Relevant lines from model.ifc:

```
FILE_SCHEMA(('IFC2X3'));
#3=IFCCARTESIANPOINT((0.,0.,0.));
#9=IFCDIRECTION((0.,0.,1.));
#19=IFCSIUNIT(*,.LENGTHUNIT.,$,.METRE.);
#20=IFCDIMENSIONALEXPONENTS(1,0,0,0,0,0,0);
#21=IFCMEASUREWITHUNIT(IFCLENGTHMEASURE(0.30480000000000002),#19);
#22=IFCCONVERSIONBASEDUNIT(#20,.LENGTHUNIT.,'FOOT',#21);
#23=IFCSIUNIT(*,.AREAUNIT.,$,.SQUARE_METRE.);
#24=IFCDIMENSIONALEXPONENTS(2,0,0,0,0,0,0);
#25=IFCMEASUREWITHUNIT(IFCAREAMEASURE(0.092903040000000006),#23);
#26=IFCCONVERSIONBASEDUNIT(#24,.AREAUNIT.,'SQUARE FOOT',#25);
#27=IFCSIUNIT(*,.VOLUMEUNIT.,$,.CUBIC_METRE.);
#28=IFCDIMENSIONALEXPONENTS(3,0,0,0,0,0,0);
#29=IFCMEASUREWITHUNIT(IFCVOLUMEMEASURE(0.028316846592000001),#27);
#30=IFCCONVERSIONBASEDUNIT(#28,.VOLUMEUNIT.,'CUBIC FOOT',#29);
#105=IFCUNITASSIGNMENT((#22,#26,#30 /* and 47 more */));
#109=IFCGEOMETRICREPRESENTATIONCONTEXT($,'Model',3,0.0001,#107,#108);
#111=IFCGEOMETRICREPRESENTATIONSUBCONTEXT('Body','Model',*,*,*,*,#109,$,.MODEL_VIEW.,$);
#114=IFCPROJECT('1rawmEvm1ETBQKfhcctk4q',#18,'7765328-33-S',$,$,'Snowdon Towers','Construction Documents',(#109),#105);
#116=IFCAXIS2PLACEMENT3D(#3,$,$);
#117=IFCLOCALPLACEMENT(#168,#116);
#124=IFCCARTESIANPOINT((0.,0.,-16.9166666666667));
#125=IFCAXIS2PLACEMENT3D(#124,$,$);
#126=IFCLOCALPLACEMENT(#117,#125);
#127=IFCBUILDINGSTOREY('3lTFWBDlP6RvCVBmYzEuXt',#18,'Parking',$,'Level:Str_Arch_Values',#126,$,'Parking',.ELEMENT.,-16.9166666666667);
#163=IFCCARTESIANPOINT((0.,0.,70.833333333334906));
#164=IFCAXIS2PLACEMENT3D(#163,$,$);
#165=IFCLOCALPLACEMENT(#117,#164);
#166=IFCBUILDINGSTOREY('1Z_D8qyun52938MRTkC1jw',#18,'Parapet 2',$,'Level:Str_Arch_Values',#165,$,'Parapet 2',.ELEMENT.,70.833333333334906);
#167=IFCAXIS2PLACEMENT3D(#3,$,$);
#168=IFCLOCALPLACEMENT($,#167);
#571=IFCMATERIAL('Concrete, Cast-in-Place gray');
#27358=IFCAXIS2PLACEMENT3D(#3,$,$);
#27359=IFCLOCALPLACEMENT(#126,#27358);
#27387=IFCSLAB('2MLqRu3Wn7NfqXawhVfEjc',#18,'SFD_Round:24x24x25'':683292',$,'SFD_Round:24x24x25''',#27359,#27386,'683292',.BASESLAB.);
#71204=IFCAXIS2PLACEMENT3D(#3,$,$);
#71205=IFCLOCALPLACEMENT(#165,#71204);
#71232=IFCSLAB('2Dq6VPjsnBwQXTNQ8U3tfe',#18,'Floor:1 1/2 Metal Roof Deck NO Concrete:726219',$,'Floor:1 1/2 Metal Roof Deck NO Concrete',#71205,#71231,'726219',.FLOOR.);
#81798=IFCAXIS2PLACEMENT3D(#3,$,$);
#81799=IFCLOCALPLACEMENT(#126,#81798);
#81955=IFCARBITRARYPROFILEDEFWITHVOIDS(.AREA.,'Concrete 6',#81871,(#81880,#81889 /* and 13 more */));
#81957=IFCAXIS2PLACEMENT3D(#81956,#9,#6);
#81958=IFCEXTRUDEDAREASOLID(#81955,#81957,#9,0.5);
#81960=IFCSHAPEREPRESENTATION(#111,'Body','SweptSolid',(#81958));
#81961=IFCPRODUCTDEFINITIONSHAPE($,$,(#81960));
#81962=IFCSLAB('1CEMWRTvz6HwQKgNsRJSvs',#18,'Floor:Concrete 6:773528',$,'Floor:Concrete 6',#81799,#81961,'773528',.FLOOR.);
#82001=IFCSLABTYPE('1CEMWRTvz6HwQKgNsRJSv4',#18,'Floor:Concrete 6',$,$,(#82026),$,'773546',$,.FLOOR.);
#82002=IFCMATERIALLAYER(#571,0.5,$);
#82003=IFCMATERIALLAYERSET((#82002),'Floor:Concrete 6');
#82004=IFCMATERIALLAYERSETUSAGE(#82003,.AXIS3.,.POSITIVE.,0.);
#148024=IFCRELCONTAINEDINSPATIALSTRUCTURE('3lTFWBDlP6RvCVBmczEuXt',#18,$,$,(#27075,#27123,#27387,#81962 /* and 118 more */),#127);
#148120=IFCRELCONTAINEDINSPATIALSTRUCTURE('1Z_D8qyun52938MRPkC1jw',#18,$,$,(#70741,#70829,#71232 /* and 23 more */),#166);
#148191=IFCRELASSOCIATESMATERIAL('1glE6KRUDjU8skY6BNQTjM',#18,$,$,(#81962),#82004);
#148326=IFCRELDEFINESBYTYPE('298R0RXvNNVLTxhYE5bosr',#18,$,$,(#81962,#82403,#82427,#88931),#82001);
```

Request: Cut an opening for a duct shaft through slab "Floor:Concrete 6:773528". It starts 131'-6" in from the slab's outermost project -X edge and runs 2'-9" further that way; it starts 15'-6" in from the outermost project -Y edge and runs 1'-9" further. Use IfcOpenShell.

```python
import numpy as np
import ifcopenshell
import ifcopenshell.api.feature
import ifcopenshell.api.geometry
import ifcopenshell.api.root
import ifcopenshell.geom
import ifcopenshell.util.placement
import ifcopenshell.util.representation
import ifcopenshell.util.shape
import ifcopenshell.util.unit

model = ifcopenshell.open("model.ifc")
unit_scale = ifcopenshell.util.unit.calculate_unit_scale(model)
settings = ifcopenshell.geom.settings()


def volume(element):
    """Net volume in cubic metres, openings subtracted."""
    shape = ifcopenshell.geom.create_shape(settings, element)
    return ifcopenshell.util.shape.get_volume(shape.geometry)


slab = model.by_id(81962)
before = volume(slab)

# Extent in the slab's own axes, in metres. The edges named are its -X and -Y sides.
slab_shape = ifcopenshell.geom.create_shape(settings, slab)
vertices = ifcopenshell.util.shape.get_vertices(slab_shape.geometry)
x_min, y_min, bottom = vertices.min(axis=0)
top = vertices[:, 2].max()

opening = ifcopenshell.api.root.create_entity(model, ifc_class="IfcOpeningElement", name="Duct shaft opening")
context = ifcopenshell.util.representation.get_context(model, "Model", "Body", "MODEL_VIEW")
width, depth = 0.8382, 0.5334
outline = [(0.0, 0.0), (width, 0.0), (width, depth), (0.0, depth), (0.0, 0.0)]
# Overshoot both faces by 50 mm so the cut is clean.
shape = ifcopenshell.api.geometry.add_slab_representation(
    model, context=context, depth=top - bottom + 0.1, polyline=outline
)
ifcopenshell.api.geometry.assign_representation(model, product=opening, representation=shape)

matrix = ifcopenshell.util.placement.get_local_placement(slab.ObjectPlacement)
matrix[:, 3] = matrix @ np.append(np.array([x_min + 40.0812, y_min + 4.7244, bottom - 0.05]) / unit_scale, 1.0)
ifcopenshell.api.geometry.edit_object_placement(model, product=opening, matrix=matrix, is_si=False)
ifcopenshell.api.feature.add_feature(model, feature=opening, element=slab)

after = volume(slab)

print(f"slab volume {before:.3f} -> {after:.3f} m3")

model.write("model-out.ifc")
```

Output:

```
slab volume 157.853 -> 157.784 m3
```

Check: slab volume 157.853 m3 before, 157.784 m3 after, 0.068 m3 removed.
